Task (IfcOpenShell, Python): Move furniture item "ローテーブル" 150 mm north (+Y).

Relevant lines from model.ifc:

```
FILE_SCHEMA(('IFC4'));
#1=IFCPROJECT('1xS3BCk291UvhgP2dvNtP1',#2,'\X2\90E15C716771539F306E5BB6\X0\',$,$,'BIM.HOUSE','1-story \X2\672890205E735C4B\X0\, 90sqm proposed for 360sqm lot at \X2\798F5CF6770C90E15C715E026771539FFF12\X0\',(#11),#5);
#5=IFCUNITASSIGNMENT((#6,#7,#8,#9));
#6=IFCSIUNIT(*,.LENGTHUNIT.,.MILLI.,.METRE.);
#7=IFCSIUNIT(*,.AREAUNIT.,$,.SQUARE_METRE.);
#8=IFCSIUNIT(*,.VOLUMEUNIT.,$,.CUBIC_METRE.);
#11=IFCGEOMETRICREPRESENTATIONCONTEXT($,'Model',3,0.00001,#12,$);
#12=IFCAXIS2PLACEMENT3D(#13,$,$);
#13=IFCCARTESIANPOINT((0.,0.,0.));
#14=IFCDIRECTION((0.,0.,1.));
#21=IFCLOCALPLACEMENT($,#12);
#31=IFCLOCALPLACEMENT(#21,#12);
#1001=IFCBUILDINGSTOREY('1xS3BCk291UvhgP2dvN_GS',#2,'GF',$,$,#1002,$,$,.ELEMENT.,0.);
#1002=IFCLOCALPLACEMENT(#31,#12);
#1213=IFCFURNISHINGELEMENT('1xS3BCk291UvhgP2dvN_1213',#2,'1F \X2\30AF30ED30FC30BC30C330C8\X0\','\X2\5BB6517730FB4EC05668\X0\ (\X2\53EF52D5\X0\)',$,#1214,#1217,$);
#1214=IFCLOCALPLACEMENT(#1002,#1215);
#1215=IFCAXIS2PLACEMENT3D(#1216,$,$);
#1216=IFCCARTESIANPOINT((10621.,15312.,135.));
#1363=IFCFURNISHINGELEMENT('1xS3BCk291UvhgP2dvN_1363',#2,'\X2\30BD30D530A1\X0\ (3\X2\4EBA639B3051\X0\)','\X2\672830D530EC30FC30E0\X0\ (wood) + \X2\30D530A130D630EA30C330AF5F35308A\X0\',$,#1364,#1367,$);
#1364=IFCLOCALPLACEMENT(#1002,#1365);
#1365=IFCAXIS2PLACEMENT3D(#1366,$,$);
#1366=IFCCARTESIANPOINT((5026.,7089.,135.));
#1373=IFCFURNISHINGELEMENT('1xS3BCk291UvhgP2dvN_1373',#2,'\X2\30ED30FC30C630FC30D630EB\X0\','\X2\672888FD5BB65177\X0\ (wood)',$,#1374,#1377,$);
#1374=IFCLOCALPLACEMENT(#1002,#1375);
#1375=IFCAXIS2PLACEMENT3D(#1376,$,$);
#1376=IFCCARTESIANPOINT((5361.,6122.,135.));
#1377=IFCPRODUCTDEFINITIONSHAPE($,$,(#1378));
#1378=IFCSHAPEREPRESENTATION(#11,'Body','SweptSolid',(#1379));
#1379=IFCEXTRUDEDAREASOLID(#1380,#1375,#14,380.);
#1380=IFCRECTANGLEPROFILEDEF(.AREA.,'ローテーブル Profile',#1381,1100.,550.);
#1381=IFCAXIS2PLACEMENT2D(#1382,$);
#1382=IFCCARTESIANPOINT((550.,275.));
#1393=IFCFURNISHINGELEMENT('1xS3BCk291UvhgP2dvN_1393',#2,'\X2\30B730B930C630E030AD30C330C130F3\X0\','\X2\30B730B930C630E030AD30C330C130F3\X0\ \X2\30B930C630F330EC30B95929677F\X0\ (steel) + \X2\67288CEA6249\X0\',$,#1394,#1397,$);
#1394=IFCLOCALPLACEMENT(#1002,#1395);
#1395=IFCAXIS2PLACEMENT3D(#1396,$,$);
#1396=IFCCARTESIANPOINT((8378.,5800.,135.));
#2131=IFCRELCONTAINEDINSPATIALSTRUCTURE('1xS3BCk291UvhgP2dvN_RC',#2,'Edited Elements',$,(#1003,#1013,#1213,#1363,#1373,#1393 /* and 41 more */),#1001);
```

```python
import ifcopenshell
import ifcopenshell.api.geometry
import ifcopenshell.util.placement

model = ifcopenshell.open("model.ifc")

item = model.by_guid("1xS3BCk291UvhgP2dvN_1373")
matrix = ifcopenshell.util.placement.get_local_placement(item.ObjectPlacement)
matrix[1, 3] += 150.0
ifcopenshell.api.geometry.edit_object_placement(model, product=item, matrix=matrix, is_si=False)

print(ifcopenshell.util.placement.get_local_placement(item.ObjectPlacement).round(3) + 0.0)

model.write("model_updated.ifc")
```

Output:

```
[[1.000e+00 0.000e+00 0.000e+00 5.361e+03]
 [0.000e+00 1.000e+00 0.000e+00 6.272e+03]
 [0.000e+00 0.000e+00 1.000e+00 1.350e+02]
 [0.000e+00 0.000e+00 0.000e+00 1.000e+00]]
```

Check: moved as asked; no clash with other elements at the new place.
